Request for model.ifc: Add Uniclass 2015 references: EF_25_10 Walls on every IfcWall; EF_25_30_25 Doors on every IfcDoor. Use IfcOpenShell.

First a look at what the model holds.

```python
import ifcopenshell

model = ifcopenshell.open("model.ifc")
print(model.schema)
print("classifications:", [c.Name for c in model.by_type("IfcClassification")])
for ifc_class in ("IfcDoor", "IfcRoof", "IfcStair", "IfcWall", "IfcWindow"):
    print(ifc_class, len(model.by_type(ifc_class)))
```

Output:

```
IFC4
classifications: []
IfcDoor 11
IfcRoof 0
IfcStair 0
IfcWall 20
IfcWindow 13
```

```python
import ifcopenshell
import ifcopenshell.api.classification

model = ifcopenshell.open("model.ifc")

system = ifcopenshell.api.classification.add_classification(model, classification="Uniclass 2015")

codes = {
    "IfcWall": ("EF_25_10", "Walls"),
    "IfcDoor": ("EF_25_30_25", "Doors"),
}
for ifc_class, (code, name) in codes.items():
    products = model.by_type(ifc_class)
    ifcopenshell.api.classification.add_reference(
        model, products=products, classification=system, identification=code, name=name
    )
    print(code, len(products))

model.write("model-out.ifc")
```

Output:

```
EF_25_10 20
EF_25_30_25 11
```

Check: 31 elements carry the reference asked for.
